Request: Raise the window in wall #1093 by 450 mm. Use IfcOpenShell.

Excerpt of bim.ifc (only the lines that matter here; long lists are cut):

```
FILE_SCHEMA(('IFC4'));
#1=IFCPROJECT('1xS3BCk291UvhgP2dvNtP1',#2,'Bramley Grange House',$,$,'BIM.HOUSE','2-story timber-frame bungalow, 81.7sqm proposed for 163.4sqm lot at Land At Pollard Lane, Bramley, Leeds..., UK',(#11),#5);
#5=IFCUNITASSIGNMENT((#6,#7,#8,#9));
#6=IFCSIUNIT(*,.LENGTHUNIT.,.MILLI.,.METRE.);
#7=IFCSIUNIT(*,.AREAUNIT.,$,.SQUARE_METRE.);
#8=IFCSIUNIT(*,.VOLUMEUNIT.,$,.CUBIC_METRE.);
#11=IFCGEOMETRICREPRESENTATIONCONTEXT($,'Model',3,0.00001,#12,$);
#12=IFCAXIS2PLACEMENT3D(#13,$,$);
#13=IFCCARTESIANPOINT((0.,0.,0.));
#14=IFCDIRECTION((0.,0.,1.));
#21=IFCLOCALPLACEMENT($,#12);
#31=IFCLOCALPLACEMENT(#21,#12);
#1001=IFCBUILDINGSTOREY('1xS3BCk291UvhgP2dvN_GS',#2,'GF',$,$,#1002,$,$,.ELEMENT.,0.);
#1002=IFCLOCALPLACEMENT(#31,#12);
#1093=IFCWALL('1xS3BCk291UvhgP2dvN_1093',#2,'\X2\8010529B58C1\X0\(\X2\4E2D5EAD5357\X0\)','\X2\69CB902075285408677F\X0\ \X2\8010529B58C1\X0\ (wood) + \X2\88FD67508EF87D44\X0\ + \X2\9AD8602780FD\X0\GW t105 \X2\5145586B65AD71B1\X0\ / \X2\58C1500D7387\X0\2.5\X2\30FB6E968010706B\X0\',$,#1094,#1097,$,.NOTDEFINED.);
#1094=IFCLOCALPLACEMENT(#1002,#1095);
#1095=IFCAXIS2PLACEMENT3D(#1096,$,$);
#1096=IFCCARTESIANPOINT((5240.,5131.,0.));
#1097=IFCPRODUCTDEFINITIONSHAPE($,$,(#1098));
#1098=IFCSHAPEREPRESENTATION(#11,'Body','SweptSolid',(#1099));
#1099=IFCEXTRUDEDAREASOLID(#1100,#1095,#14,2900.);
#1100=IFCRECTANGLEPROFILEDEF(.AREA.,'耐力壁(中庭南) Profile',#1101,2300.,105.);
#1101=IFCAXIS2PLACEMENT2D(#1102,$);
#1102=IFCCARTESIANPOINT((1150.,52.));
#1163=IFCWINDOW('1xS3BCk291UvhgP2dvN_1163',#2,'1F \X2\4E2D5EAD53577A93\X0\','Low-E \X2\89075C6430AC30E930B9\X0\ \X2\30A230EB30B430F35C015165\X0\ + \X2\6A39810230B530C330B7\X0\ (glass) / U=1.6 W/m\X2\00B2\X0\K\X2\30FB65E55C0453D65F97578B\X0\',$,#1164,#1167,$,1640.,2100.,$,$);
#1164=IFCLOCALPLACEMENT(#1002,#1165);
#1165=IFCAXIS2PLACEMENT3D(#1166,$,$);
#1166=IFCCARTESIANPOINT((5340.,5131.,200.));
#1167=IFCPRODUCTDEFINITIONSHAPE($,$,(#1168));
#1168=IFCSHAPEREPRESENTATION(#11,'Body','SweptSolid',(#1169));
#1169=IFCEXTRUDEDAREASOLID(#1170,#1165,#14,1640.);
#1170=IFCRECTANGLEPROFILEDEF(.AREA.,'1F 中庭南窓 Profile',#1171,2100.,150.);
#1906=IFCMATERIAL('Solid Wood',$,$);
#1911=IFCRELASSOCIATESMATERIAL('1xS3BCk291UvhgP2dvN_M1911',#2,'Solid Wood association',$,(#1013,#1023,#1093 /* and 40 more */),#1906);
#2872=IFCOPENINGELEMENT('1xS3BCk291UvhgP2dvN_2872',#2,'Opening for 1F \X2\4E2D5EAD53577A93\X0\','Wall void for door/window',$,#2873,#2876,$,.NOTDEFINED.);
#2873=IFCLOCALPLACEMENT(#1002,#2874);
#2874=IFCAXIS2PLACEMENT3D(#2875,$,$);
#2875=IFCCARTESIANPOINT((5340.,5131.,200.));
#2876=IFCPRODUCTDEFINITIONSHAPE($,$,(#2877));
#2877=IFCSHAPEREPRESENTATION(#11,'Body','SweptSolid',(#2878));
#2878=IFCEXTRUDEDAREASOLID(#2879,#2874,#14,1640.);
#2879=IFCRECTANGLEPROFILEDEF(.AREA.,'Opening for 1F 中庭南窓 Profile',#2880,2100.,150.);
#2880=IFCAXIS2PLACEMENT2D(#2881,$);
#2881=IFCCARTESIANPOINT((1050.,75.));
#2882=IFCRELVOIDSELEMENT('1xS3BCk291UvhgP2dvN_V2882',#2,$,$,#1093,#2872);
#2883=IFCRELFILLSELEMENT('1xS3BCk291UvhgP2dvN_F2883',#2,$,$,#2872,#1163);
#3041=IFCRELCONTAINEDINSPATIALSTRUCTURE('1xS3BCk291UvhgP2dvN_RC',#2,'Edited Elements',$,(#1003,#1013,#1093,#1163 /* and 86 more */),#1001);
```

```python
import numpy as np
import ifcopenshell
import ifcopenshell.api.geometry
import ifcopenshell.util.placement
import ifcopenshell.util.unit

model = ifcopenshell.open("bim.ifc")
unit_scale = ifcopenshell.util.unit.calculate_unit_scale(model)

window = model.by_guid("1xS3BCk291UvhgP2dvN_1163")
opening = window.FillsVoids[0].RelatingOpeningElement
dz = 0.45 / unit_scale

shift = np.array([0.0, 0.0, dz])
# The window is not placed relative to its opening, so move both.
for product in (opening, window):
    matrix = ifcopenshell.util.placement.get_local_placement(product.ObjectPlacement)
    matrix[:3, 3] += shift
    ifcopenshell.api.geometry.edit_object_placement(model, product=product, matrix=matrix, is_si=False)

print(f"moved by {dz * unit_scale:+.3f} m")

model.write("bim_updated.ifc")
```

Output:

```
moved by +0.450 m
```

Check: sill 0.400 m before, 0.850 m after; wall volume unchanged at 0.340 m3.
